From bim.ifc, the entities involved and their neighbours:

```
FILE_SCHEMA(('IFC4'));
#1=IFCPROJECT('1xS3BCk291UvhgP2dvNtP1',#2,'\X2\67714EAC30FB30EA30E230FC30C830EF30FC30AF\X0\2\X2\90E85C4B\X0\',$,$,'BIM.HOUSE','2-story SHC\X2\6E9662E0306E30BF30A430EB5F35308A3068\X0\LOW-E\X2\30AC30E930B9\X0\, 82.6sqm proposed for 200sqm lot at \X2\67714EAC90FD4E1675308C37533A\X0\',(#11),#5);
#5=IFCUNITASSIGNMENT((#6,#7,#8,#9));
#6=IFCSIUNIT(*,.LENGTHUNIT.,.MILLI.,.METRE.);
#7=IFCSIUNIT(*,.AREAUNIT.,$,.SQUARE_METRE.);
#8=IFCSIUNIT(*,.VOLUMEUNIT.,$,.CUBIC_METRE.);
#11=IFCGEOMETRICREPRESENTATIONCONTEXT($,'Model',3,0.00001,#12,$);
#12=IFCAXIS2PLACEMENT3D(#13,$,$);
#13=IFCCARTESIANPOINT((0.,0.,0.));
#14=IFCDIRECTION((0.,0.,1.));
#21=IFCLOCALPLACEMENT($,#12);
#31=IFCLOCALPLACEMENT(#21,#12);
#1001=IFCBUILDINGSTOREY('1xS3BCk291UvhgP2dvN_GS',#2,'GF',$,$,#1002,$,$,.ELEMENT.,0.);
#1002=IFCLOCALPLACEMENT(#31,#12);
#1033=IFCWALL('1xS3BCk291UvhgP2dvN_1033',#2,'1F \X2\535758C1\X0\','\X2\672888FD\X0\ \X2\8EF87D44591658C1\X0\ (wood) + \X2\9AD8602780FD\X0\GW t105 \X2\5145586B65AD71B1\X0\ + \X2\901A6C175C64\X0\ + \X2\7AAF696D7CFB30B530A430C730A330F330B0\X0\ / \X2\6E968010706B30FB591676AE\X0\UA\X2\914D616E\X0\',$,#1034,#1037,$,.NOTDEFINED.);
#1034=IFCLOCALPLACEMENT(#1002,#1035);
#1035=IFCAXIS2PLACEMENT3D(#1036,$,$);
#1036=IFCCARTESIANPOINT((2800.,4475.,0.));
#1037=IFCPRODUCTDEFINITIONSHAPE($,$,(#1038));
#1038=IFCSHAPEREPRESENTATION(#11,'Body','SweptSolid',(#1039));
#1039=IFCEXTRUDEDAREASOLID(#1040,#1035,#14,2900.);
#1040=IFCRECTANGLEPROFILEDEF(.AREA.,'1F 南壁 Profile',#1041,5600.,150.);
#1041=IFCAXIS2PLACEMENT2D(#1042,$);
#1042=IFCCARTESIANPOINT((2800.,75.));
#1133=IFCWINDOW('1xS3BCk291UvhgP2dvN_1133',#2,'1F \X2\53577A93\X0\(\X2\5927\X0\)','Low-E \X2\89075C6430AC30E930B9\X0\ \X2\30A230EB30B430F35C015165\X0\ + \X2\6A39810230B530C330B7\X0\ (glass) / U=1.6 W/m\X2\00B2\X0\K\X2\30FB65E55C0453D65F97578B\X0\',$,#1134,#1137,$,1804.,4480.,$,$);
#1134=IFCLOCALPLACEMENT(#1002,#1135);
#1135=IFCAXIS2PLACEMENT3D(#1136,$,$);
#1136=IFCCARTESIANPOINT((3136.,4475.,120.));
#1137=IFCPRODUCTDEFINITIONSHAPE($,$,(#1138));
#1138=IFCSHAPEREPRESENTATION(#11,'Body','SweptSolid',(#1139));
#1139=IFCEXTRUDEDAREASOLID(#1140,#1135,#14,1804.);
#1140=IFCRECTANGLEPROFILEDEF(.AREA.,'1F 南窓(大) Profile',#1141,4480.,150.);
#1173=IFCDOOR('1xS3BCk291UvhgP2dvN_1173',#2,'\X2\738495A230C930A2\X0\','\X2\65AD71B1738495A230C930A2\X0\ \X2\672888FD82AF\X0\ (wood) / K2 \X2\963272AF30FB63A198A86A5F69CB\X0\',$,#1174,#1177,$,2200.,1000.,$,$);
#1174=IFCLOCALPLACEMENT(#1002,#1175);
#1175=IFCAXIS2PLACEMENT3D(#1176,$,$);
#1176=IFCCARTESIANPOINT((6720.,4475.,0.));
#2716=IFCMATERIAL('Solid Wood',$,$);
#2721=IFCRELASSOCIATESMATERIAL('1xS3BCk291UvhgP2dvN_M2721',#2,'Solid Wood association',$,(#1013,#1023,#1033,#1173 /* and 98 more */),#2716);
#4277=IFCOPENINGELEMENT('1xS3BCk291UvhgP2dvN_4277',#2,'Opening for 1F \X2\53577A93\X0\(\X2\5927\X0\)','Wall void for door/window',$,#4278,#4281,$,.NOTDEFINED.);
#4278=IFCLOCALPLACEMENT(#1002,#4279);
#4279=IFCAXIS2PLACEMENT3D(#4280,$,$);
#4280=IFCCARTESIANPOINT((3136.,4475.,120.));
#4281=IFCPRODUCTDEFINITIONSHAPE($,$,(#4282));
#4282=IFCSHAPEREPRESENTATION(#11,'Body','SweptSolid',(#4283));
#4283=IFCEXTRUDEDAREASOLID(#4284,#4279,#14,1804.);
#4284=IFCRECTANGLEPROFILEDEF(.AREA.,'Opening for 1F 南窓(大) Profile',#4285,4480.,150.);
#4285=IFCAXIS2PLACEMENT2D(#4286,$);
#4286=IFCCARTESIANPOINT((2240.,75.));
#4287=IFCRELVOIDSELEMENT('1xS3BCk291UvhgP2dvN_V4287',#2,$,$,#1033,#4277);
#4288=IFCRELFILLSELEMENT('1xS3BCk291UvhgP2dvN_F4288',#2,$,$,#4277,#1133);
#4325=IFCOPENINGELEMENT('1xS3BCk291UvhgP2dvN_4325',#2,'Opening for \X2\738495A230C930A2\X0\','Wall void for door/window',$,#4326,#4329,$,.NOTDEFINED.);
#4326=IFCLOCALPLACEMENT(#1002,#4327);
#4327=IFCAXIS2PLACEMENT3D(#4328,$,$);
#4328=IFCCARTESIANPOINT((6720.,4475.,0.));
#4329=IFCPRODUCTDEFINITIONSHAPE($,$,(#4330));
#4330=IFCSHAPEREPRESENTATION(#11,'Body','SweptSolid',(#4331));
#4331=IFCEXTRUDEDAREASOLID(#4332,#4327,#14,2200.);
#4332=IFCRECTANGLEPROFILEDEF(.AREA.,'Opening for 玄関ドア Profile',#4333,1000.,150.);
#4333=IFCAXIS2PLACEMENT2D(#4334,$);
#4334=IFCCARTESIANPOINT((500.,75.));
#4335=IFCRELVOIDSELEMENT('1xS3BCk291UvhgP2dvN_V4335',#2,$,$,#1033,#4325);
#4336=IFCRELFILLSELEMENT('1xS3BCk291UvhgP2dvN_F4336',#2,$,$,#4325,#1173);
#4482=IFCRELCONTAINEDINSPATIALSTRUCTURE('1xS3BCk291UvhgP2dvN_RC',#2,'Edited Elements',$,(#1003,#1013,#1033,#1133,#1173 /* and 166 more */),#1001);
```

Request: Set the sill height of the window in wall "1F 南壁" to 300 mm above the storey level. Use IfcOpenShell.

```python
import numpy as np
import ifcopenshell
import ifcopenshell.api.geometry
import ifcopenshell.geom
import ifcopenshell.util.element
import ifcopenshell.util.placement
import ifcopenshell.util.shape
import ifcopenshell.util.unit

model = ifcopenshell.open("bim.ifc")
unit_scale = ifcopenshell.util.unit.calculate_unit_scale(model)

window = model.by_guid("1xS3BCk291UvhgP2dvN_1133")
opening = window.FillsVoids[0].RelatingOpeningElement
storey = ifcopenshell.util.element.get_container(window, ifc_class="IfcBuildingStorey")
level = ifcopenshell.util.placement.get_local_placement(storey.ObjectPlacement)[2, 3]

# The opening's origin need not be at the sill, so measure its lowest point.
shape = ifcopenshell.geom.create_shape(ifcopenshell.geom.settings(), opening)
bottom = ifcopenshell.util.shape.get_shape_bottom_elevation(shape, shape.geometry) / unit_scale
dz = level + 0.3 / unit_scale - bottom

shift = np.array([0.0, 0.0, dz])
# The window is not placed relative to its opening, so move both.
for product in (opening, window):
    matrix = ifcopenshell.util.placement.get_local_placement(product.ObjectPlacement)
    matrix[:3, 3] += shift
    ifcopenshell.api.geometry.edit_object_placement(model, product=product, matrix=matrix, is_si=False)

print(f"moved by {dz * unit_scale:+.3f} m")

model.write("bim_edited.ifc")
```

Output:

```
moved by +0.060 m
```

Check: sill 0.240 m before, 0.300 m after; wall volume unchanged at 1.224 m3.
